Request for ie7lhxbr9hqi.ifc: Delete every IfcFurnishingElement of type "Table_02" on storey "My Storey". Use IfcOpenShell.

First a look at what the model holds.

```python
import ifcopenshell
import ifcopenshell.util.element

model = ifcopenshell.open("ie7lhxbr9hqi.ifc")
print(model.schema)
storey = next(s for s in model.by_type("IfcBuildingStorey") if s.Name == "My Storey")
furniture = [e for e in ifcopenshell.util.element.get_decomposition(storey) if e.is_a("IfcFurnishingElement")]
seen = {}
for e in furniture:
    element_type = ifcopenshell.util.element.get_type(e)
    name = element_type.Name if element_type not in (None, e) else None
    seen[name] = seen.get(name, 0) + 1
for name, count in sorted(seen.items(), key=str):
    print(count, "x", name)
```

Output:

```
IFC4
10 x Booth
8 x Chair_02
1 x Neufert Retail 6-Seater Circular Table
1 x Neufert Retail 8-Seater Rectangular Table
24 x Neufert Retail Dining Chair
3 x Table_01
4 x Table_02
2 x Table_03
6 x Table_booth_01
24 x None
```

```python
import ifcopenshell
import ifcopenshell.api.root
import ifcopenshell.util.element

model = ifcopenshell.open("ie7lhxbr9hqi.ifc")

storey = next(s for s in model.by_type("IfcBuildingStorey") if s.Name == "My Storey")
furniture = [e for e in ifcopenshell.util.element.get_decomposition(storey) if e.is_a("IfcFurnishingElement")]
targets = [e for e in furniture if (t := ifcopenshell.util.element.get_type(e)) not in (None, e) and t.Name == "Table_02"]

for e in targets:
    ifcopenshell.api.root.remove_product(model, product=e)
print(len(targets), "removed")

model.write("ie7lhxbr9hqi_v2.ifc")
```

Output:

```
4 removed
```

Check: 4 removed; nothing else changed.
